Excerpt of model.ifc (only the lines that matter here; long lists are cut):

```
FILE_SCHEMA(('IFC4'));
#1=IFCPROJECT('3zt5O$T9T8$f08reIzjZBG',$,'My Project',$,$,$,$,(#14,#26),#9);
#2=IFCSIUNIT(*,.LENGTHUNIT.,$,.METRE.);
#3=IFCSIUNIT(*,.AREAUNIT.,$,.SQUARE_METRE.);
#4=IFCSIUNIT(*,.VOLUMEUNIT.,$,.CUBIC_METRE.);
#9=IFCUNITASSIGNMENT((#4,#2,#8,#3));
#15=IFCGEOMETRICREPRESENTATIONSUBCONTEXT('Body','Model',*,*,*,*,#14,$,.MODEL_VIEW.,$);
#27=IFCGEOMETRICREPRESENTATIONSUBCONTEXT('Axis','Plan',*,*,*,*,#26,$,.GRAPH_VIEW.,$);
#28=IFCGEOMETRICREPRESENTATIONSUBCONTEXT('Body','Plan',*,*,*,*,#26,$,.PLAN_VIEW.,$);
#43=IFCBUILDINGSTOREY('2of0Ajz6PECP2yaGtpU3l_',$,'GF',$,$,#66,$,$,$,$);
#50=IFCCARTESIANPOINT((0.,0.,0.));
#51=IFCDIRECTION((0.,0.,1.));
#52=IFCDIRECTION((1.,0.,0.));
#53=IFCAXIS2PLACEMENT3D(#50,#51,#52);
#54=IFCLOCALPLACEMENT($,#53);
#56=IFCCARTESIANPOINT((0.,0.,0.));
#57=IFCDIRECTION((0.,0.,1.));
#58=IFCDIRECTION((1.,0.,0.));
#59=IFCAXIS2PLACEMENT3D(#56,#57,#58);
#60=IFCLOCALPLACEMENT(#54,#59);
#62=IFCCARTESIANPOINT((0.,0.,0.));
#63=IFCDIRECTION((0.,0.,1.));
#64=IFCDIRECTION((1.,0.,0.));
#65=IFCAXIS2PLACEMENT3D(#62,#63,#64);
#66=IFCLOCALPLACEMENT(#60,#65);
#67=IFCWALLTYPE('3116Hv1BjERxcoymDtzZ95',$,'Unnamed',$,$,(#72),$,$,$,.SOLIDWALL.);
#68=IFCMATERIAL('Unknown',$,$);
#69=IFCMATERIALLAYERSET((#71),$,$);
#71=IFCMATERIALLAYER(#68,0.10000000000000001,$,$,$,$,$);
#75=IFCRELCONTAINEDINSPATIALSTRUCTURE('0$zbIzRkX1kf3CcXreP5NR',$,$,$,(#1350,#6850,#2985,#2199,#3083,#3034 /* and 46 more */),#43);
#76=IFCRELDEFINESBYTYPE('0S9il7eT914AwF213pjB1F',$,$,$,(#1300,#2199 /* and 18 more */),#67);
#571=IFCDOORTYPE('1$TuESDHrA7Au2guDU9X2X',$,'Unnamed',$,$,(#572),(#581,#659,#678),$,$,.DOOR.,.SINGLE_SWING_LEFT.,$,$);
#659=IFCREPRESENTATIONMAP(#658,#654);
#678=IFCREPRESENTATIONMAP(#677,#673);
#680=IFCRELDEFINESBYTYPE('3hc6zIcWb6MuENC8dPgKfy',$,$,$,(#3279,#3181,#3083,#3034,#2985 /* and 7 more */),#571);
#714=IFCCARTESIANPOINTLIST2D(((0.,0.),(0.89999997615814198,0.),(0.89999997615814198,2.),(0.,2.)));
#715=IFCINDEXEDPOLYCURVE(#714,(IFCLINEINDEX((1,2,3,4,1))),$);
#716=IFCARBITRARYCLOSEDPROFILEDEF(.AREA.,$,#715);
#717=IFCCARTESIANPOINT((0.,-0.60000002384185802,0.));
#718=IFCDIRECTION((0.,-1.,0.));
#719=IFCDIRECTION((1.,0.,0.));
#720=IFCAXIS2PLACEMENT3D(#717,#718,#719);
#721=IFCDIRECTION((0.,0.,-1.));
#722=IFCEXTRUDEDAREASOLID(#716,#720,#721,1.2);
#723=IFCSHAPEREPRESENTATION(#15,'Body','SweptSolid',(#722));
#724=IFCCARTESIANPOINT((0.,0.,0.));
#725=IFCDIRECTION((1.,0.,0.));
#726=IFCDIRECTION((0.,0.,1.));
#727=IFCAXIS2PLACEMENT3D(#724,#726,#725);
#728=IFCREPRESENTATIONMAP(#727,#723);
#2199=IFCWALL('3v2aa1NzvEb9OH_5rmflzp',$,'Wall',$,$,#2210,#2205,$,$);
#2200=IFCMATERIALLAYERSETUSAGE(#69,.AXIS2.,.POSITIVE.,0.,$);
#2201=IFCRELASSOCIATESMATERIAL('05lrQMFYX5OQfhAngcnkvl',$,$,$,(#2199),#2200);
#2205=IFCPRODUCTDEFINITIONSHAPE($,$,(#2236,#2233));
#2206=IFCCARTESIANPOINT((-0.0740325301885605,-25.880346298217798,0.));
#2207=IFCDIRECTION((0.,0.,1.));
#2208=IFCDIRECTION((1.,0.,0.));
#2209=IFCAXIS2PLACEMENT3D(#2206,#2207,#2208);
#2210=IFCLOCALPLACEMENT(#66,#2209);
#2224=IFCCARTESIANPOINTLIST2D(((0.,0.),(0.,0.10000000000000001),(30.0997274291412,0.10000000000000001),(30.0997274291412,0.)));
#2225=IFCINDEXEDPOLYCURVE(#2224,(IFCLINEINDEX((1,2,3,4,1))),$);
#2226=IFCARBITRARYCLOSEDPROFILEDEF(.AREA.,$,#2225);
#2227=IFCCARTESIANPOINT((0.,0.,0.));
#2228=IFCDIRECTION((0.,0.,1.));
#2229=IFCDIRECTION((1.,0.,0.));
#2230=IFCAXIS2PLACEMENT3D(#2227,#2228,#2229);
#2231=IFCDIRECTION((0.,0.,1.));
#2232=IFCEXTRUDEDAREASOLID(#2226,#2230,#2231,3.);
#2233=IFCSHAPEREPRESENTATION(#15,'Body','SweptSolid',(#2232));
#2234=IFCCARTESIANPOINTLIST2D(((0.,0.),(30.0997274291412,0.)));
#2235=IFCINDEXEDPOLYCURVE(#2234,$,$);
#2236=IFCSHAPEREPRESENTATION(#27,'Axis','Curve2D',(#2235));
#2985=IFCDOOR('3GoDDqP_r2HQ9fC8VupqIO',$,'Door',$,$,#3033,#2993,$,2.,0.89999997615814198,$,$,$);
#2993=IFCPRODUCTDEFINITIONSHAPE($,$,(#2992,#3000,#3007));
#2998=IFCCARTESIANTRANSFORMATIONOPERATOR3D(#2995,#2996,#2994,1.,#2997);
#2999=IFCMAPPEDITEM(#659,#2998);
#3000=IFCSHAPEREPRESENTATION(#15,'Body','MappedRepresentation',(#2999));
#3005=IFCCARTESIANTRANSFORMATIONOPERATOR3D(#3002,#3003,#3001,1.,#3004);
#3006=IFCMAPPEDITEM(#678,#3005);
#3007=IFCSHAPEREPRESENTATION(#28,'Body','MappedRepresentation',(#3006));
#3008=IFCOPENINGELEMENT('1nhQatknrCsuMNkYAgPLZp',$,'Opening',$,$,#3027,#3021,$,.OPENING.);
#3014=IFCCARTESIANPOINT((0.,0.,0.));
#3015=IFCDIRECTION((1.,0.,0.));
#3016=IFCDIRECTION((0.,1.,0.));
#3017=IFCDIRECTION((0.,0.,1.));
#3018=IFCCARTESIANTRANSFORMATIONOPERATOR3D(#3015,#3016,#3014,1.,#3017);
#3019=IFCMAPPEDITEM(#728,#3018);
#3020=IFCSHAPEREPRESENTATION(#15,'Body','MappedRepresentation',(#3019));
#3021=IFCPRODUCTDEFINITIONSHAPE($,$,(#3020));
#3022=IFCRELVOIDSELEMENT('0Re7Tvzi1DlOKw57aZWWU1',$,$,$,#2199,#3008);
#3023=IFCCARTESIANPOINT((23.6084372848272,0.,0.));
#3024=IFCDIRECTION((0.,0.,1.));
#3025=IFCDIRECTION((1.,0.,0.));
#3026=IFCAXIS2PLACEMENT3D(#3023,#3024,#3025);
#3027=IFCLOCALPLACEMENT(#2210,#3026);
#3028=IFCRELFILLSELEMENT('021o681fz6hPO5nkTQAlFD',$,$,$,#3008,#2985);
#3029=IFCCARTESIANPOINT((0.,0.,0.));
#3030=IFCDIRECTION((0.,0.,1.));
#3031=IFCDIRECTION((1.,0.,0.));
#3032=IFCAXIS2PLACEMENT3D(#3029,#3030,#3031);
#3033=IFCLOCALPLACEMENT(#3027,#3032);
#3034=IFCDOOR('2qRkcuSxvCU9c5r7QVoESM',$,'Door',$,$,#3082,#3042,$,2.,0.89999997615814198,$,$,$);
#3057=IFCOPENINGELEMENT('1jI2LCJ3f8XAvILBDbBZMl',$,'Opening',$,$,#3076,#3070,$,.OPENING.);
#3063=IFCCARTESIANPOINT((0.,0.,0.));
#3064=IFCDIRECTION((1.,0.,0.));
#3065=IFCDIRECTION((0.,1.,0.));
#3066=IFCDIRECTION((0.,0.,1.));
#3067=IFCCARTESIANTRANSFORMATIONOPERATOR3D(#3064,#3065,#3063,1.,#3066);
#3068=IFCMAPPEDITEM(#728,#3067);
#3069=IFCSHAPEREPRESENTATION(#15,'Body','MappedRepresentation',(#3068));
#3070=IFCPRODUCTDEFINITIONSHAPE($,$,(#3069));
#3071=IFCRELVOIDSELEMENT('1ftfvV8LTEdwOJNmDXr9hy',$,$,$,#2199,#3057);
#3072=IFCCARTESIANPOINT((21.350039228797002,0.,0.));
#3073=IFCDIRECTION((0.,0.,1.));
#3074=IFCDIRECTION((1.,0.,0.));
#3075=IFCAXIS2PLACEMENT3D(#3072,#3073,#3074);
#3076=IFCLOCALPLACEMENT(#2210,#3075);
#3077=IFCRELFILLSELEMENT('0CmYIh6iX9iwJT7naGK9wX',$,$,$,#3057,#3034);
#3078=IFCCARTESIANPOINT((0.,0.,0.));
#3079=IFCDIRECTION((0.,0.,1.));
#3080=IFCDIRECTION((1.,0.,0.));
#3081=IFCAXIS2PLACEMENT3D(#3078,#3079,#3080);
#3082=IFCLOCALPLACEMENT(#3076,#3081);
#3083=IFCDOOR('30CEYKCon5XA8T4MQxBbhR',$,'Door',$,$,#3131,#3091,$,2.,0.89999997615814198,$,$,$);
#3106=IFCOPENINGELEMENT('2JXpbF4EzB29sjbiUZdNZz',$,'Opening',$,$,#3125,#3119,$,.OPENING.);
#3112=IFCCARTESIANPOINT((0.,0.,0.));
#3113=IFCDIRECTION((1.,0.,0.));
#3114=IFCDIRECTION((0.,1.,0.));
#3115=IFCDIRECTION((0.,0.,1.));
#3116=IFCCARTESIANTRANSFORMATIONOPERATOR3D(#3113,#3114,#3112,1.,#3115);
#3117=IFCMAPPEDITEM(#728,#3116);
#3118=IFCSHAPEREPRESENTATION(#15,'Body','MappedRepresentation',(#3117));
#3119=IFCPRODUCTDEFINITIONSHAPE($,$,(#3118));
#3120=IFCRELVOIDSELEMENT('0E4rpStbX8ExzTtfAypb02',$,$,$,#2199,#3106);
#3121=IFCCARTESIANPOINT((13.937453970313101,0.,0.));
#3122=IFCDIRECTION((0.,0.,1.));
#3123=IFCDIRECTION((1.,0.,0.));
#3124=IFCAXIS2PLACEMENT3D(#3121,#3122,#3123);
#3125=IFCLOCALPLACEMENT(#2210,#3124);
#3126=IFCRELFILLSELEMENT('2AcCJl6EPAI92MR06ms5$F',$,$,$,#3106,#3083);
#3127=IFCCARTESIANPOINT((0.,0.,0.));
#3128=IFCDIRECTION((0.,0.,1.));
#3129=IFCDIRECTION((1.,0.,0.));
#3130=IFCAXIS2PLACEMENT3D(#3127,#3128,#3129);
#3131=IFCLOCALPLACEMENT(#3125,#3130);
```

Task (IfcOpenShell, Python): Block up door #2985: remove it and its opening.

```python
import ifcopenshell
import ifcopenshell.api.feature
import ifcopenshell.api.root
import ifcopenshell.geom
import ifcopenshell.util.shape

model = ifcopenshell.open("model.ifc")
settings = ifcopenshell.geom.settings()


def volume(element):
    """Net volume in cubic metres, openings subtracted."""
    shape = ifcopenshell.geom.create_shape(settings, element)
    return ifcopenshell.util.shape.get_volume(shape.geometry)


door = model.by_guid("3GoDDqP_r2HQ9fC8VupqIO")
opening = door.FillsVoids[0].RelatingOpeningElement
wall = opening.VoidsElements[0].RelatingBuildingElement
before = volume(wall)

ifcopenshell.api.root.remove_product(model, product=door)
ifcopenshell.api.feature.remove_feature(model, feature=opening)

after = volume(wall)

print(f"wall volume {before:.3f} -> {after:.3f} m3")

model.write("model_v2.ifc")
```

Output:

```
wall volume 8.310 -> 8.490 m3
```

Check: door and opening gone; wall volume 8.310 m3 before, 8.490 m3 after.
